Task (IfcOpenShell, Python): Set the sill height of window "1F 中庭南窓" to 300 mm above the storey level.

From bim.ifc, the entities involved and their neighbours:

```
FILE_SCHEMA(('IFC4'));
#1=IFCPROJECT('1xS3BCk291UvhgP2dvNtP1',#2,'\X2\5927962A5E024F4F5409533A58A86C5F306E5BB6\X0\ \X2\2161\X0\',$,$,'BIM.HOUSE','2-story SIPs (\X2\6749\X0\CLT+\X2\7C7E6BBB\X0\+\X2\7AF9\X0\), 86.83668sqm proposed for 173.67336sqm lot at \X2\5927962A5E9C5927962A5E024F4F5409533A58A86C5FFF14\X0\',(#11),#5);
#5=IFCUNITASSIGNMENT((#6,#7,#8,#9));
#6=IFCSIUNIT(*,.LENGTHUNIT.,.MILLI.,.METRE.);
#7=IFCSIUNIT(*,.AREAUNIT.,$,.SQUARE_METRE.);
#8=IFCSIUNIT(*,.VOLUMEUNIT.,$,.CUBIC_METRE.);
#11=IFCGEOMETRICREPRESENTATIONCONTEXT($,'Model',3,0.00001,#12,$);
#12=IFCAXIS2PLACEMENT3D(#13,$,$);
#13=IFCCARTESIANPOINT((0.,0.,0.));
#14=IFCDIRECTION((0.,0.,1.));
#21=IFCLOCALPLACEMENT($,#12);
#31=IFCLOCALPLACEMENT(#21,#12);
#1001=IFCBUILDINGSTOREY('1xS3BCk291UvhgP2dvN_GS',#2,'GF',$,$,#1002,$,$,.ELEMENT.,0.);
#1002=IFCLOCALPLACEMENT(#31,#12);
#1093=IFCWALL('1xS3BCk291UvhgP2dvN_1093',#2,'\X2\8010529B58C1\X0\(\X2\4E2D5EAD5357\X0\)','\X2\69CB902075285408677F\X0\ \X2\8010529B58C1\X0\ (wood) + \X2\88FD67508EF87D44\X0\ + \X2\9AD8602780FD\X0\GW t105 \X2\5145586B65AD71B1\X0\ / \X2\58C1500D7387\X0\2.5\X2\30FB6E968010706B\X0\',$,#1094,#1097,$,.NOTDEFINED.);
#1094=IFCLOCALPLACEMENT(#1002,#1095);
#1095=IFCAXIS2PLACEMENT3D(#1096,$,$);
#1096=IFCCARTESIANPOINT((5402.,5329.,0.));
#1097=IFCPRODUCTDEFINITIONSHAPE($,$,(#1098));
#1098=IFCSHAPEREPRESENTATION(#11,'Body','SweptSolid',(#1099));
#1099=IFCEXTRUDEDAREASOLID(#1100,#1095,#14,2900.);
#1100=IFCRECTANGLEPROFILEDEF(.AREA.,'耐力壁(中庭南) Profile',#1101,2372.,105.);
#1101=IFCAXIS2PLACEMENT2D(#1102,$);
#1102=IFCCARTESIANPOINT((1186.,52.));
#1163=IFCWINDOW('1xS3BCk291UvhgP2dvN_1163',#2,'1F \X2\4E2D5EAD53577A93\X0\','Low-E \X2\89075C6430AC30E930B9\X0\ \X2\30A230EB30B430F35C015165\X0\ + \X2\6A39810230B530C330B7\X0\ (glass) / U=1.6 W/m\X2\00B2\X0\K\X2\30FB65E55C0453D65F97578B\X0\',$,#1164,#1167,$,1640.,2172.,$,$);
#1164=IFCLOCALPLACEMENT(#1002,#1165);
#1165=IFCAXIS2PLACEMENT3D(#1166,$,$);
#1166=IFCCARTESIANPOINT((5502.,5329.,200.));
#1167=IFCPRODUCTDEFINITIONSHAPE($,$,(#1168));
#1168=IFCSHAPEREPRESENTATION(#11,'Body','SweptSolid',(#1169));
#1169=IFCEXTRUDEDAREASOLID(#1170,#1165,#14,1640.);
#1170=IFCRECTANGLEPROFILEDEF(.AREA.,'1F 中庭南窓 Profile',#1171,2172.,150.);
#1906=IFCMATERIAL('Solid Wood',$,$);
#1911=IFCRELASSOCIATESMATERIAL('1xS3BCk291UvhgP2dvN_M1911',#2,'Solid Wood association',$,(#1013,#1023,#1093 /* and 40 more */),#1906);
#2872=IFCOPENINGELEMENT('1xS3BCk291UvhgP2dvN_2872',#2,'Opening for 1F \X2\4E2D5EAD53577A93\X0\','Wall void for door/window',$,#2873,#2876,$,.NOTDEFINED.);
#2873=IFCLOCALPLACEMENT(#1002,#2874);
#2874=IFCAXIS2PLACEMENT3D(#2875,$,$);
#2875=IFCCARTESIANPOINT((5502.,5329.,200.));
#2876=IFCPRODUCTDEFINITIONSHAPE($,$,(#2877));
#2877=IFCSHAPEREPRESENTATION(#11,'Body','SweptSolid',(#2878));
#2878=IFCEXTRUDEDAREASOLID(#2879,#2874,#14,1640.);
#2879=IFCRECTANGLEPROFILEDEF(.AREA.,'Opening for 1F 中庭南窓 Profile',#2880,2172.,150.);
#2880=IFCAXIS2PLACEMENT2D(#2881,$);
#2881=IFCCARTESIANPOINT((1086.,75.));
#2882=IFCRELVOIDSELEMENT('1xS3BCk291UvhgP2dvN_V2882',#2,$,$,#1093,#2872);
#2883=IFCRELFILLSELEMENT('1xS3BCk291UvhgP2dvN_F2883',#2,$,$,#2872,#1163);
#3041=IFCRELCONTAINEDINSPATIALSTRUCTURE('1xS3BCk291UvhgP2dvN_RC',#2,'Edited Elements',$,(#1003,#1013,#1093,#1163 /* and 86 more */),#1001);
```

```python
import numpy as np
import ifcopenshell
import ifcopenshell.api.geometry
import ifcopenshell.geom
import ifcopenshell.util.element
import ifcopenshell.util.placement
import ifcopenshell.util.shape
import ifcopenshell.util.unit

model = ifcopenshell.open("bim.ifc")
unit_scale = ifcopenshell.util.unit.calculate_unit_scale(model)

window = model.by_guid("1xS3BCk291UvhgP2dvN_1163")
opening = window.FillsVoids[0].RelatingOpeningElement
storey = ifcopenshell.util.element.get_container(window, ifc_class="IfcBuildingStorey")
level = ifcopenshell.util.placement.get_local_placement(storey.ObjectPlacement)[2, 3]

# The opening's origin need not be at the sill, so measure its lowest point.
shape = ifcopenshell.geom.create_shape(ifcopenshell.geom.settings(), opening)
bottom = ifcopenshell.util.shape.get_shape_bottom_elevation(shape, shape.geometry) / unit_scale
dz = level + 0.3 / unit_scale - bottom

shift = np.array([0.0, 0.0, dz])
# The window is not placed relative to its opening, so move both.
for product in (opening, window):
    matrix = ifcopenshell.util.placement.get_local_placement(product.ObjectPlacement)
    matrix[:3, 3] += shift
    ifcopenshell.api.geometry.edit_object_placement(model, product=product, matrix=matrix, is_si=False)

print(f"moved by {dz * unit_scale:+.3f} m")

model.write("bim_updated.ifc")
```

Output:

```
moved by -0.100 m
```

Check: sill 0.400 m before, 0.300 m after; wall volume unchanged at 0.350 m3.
